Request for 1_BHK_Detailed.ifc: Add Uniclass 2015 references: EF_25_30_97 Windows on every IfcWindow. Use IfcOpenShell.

First a look at what the model holds.

```python
import ifcopenshell

model = ifcopenshell.open("1_BHK_Detailed.ifc")
print(model.schema)
print("classifications:", [c.Name for c in model.by_type("IfcClassification")])
for ifc_class in ("IfcDoor", "IfcRoof", "IfcStair", "IfcWall", "IfcWindow"):
    print(ifc_class, len(model.by_type(ifc_class)))
```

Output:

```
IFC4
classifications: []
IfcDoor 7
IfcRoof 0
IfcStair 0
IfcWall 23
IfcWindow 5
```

```python
import ifcopenshell
import ifcopenshell.api.classification

model = ifcopenshell.open("1_BHK_Detailed.ifc")

system = ifcopenshell.api.classification.add_classification(model, classification="Uniclass 2015")

codes = {
    "IfcWindow": ("EF_25_30_97", "Windows"),
}
for ifc_class, (code, name) in codes.items():
    products = model.by_type(ifc_class)
    ifcopenshell.api.classification.add_reference(
        model, products=products, classification=system, identification=code, name=name
    )
    print(code, len(products))

model.write("1_BHK_Detailed_edited.ifc")
```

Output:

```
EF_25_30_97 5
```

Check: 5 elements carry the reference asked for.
